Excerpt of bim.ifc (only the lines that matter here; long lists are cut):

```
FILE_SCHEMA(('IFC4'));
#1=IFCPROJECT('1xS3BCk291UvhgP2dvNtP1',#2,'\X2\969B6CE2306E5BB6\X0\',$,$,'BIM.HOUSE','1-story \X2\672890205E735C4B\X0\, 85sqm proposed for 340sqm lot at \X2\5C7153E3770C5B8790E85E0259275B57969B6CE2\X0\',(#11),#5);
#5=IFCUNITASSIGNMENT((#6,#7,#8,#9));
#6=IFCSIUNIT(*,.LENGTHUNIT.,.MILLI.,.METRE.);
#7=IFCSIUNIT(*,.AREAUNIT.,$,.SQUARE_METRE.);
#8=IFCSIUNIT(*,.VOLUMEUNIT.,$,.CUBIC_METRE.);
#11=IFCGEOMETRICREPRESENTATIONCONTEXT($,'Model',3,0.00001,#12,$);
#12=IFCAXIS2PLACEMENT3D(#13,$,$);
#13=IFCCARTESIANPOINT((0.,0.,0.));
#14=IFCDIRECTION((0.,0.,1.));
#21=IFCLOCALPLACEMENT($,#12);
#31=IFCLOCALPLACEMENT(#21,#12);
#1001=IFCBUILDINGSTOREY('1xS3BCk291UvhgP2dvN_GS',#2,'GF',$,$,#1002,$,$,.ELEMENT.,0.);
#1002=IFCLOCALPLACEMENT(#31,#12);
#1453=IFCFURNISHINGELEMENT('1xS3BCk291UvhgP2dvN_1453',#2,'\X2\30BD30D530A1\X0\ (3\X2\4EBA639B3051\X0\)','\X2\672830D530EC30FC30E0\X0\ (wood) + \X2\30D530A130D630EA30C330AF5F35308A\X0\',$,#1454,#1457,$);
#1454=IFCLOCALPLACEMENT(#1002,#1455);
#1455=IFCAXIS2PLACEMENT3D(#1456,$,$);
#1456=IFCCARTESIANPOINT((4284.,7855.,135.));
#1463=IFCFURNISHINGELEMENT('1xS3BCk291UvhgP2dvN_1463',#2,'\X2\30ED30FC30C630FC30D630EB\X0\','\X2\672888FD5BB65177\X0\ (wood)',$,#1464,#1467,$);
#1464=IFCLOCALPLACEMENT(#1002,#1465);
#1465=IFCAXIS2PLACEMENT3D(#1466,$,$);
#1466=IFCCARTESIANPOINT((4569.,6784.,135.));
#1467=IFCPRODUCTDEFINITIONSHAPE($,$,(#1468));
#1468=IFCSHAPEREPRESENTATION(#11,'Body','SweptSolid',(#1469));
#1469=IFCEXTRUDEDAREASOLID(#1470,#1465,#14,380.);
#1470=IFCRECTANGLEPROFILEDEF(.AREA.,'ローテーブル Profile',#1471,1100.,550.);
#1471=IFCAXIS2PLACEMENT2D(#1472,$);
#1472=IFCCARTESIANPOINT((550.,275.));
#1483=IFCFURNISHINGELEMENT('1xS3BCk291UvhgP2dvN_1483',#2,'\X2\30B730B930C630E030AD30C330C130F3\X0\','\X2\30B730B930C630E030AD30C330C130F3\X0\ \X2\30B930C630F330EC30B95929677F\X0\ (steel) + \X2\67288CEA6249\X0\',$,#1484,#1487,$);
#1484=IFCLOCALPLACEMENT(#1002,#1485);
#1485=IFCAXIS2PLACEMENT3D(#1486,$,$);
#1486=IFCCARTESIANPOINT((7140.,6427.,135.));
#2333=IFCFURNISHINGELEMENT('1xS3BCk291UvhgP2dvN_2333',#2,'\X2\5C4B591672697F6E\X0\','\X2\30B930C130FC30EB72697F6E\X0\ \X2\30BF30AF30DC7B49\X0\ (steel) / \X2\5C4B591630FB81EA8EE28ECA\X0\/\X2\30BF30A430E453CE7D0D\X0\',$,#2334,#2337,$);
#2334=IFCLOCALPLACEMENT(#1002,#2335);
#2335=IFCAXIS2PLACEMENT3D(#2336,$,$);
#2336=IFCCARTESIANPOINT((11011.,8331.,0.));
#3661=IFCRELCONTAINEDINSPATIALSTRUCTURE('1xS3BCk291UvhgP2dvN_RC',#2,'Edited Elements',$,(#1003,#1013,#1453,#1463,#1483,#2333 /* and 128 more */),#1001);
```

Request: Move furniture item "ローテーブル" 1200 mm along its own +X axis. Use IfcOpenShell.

```python
import ifcopenshell
import ifcopenshell.api.geometry
import ifcopenshell.util.placement
import ifcopenshell.util.unit

model = ifcopenshell.open("bim.ifc")
unit_scale = ifcopenshell.util.unit.calculate_unit_scale(model)

item = model.by_id(1463)
matrix = ifcopenshell.util.placement.get_local_placement(item.ObjectPlacement)
matrix[:3, 3] += matrix[:3, 0] * 1.2 / unit_scale
ifcopenshell.api.geometry.edit_object_placement(model, product=item, matrix=matrix, is_si=False)

print(ifcopenshell.util.placement.get_local_placement(item.ObjectPlacement).round(3) + 0.0)

model.write("bim-out.ifc")
```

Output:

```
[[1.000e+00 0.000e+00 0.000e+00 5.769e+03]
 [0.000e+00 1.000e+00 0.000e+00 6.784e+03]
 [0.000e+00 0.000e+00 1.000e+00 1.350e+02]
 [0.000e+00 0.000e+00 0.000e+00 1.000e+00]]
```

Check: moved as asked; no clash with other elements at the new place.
